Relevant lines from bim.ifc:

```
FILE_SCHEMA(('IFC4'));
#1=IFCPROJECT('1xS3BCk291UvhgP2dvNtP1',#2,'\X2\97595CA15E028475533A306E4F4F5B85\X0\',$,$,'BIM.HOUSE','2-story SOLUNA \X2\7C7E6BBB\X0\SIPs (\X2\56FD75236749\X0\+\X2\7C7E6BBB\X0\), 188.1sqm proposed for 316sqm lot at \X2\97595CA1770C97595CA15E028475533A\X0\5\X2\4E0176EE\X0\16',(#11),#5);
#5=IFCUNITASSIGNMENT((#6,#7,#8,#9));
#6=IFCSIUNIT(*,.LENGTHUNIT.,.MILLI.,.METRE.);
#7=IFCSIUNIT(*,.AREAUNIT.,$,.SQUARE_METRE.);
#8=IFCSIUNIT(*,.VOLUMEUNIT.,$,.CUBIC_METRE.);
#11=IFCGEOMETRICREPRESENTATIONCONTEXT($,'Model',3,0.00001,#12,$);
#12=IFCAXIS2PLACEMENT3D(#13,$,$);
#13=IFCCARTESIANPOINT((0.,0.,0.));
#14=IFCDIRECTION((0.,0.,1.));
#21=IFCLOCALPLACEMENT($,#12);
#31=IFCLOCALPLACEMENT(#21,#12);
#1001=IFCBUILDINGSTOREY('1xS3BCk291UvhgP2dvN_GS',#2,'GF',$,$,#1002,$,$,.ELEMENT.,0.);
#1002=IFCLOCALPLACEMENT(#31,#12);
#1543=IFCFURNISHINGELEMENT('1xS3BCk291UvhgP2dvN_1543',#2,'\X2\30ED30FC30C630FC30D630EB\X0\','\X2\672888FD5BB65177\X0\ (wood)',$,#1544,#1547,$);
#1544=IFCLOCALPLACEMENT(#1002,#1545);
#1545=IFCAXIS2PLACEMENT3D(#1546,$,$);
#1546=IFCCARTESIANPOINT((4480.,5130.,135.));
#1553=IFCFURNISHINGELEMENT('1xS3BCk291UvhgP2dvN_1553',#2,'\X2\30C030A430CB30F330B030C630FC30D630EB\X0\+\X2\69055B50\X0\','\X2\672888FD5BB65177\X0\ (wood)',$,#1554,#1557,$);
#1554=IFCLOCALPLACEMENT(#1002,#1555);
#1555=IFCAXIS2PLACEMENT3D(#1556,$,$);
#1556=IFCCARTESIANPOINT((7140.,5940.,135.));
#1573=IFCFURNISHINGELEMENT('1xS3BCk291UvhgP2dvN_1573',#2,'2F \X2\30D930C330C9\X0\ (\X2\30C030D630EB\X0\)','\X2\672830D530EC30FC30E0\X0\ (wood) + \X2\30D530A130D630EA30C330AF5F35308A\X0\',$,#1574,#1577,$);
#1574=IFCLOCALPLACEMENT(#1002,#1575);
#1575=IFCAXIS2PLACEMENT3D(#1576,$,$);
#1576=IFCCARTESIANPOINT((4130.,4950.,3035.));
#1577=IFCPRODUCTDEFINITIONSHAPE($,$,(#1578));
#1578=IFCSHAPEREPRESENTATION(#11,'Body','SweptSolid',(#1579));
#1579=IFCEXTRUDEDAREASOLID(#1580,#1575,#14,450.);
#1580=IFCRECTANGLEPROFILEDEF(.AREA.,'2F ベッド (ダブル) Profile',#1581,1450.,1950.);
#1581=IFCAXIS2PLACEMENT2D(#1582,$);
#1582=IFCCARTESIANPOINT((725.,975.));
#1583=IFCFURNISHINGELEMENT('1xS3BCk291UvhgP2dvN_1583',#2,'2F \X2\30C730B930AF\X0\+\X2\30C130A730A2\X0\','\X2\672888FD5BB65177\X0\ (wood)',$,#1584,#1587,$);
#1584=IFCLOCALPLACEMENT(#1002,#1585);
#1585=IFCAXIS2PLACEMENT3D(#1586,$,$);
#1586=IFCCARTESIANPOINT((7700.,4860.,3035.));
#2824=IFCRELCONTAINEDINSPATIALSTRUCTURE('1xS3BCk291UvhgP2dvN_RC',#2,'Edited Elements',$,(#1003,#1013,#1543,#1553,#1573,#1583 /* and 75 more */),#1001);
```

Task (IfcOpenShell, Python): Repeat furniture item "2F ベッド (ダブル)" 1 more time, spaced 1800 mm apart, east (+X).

```python
import numpy as np
import ifcopenshell
import ifcopenshell.api.geometry
import ifcopenshell.api.root
import ifcopenshell.util.element
import ifcopenshell.util.placement

model = ifcopenshell.open("bim.ifc")


def reuse_history(source, copy):
    """copy_class also copies each property set's owner history, people and application; keep the originals."""
    for rel in copy.IsDefinedBy:
        if rel.is_a("IfcRelDefinesByProperties") and (history := rel.RelatingPropertyDefinition.OwnerHistory):
            rel.RelatingPropertyDefinition.OwnerHistory = source.OwnerHistory
            ifcopenshell.util.element.remove_deep2(model, history)


source = model.by_id(1573)
base = ifcopenshell.util.placement.get_local_placement(source.ObjectPlacement)
step = np.array([1.0, 0.0, 0.0]) * 1800.0

for i in range(1, 2):
    copy = ifcopenshell.api.root.copy_class(model, product=source)
    copy.Representation = ifcopenshell.util.element.copy_deep(
        model, source.Representation, exclude=["IfcGeometricRepresentationContext", "IfcRepresentationMap"]
    )
    reuse_history(source, copy)
    matrix = base.copy()
    matrix[:3, 3] += i * step
    print("added at", matrix[:3, 3].round(3) + 0.0)
    ifcopenshell.api.geometry.edit_object_placement(model, product=copy, matrix=matrix, is_si=False)

model.write("bim_v2.ifc")
```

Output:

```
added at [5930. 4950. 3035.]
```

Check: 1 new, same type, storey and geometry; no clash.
